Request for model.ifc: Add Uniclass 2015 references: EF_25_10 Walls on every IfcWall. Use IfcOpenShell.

First a look at what the model holds.

```python
import ifcopenshell

model = ifcopenshell.open("model.ifc")
print(model.schema)
print("classifications:", [c.Name for c in model.by_type("IfcClassification")])
for ifc_class in ("IfcDoor", "IfcRoof", "IfcStair", "IfcWall", "IfcWindow"):
    print(ifc_class, len(model.by_type(ifc_class)))
```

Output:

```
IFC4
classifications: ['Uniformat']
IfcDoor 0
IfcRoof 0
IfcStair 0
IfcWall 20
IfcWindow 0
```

```python
import ifcopenshell
import ifcopenshell.api.classification

model = ifcopenshell.open("model.ifc")

system = ifcopenshell.api.classification.add_classification(model, classification="Uniclass 2015")

codes = {
    "IfcWall": ("EF_25_10", "Walls"),
}
for ifc_class, (code, name) in codes.items():
    products = model.by_type(ifc_class)
    ifcopenshell.api.classification.add_reference(
        model, products=products, classification=system, identification=code, name=name
    )
    print(code, len(products))

model.write("model_rev.ifc")
```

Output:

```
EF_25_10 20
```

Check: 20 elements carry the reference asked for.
